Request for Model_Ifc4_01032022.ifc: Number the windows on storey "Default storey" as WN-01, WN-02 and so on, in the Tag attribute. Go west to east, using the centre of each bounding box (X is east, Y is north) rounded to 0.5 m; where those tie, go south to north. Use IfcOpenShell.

First a look at what the model holds.

```python
import ifcopenshell
import ifcopenshell.util.element
import ifcopenshell.util.placement

model = ifcopenshell.open("Model_Ifc4_01032022.ifc")
print(model.schema)
storey = next(s for s in model.by_type("IfcBuildingStorey") if s.Name == "Default storey")
windows = [e for e in ifcopenshell.util.element.get_decomposition(storey) if e.is_a("IfcWindow")]
for e in sorted(windows, key=lambda e: e.id()):
    origin = ifcopenshell.util.placement.get_local_placement(e.ObjectPlacement)[:3, 3]
    print(e.id(), e.Tag, e.Name, origin.round(2) + 0.0, sep=" | ")
```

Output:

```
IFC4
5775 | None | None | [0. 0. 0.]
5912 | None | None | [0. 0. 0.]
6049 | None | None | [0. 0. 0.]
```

```python
import ifcopenshell
import ifcopenshell.geom
import ifcopenshell.util.element
import ifcopenshell.util.shape

model = ifcopenshell.open("Model_Ifc4_01032022.ifc")
settings = ifcopenshell.geom.settings()
settings.set("use-world-coords", True)


def centre(element):
    shape = ifcopenshell.geom.create_shape(settings, element)
    return ifcopenshell.util.shape.get_bbox_centroid(shape.geometry)


storey = next(s for s in model.by_type("IfcBuildingStorey") if s.Name == "Default storey")
windows = [e for e in ifcopenshell.util.element.get_decomposition(storey) if e.is_a("IfcWindow")]

# Insertion points can sit at a corner or the storey origin, so sort by the geometry (in metres).
centres = {e: centre(e) for e in windows}
windows.sort(key=lambda e: (round(centres[e][0] / 0.5), centres[e][1]))

for i, e in enumerate(windows, start=1):
    number = f"WN-{i:02d}"
    e.Tag = number
    print(e.id(), number)

model.write("Model_Ifc4_01032022_edited.ifc")
```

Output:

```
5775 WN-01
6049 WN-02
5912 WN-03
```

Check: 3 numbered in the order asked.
